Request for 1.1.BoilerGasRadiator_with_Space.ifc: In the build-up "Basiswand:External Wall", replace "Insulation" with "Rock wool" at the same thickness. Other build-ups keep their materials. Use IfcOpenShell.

First a look at what the model holds.

```python
import ifcopenshell
import ifcopenshell.util.element

model = ifcopenshell.open("1.1.BoilerGasRadiator_with_Space.ifc")
print(model.schema)
for layer_set in model.by_type("IfcMaterialLayerSet"):
    if layer_set.LayerSetName == "Basiswand:External Wall":
        for layer in layer_set.MaterialLayers:
            print(layer.id(), layer.Material and layer.Material.Name, layer.LayerThickness, sep=" | ")
        print(len(ifcopenshell.util.element.get_elements_by_material(model, layer_set)), "elements and types use it")
print(sorted(m.Name for m in model.by_type("IfcMaterial") if m.Name)[:60])
```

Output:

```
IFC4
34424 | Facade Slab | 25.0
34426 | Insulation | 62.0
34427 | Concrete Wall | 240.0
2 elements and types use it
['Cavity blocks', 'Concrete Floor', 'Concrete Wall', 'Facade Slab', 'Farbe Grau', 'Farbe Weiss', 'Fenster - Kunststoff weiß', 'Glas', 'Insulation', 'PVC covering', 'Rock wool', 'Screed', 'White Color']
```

```python
import ifcopenshell
import ifcopenshell.api.material

model = ifcopenshell.open("1.1.BoilerGasRadiator_with_Space.ifc")

layer_set = next(s for s in model.by_type("IfcMaterialLayerSet") if s.LayerSetName == "Basiswand:External Wall")
layer = next(l for l in layer_set.MaterialLayers if l.Material and l.Material.Name == "Insulation")
material = next(m for m in model.by_type("IfcMaterial") if m.Name == "Rock wool")

# Point this one layer at the other material; renaming the old one would change it everywhere.
ifcopenshell.api.material.edit_layer(model, layer=layer, attributes={}, material=material)

print([l.Material.Name if l.Material else None for l in layer_set.MaterialLayers])

model.write("1.1.BoilerGasRadiator_with_Space_edited.ifc")
```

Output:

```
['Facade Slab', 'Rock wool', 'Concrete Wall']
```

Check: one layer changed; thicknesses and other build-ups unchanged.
